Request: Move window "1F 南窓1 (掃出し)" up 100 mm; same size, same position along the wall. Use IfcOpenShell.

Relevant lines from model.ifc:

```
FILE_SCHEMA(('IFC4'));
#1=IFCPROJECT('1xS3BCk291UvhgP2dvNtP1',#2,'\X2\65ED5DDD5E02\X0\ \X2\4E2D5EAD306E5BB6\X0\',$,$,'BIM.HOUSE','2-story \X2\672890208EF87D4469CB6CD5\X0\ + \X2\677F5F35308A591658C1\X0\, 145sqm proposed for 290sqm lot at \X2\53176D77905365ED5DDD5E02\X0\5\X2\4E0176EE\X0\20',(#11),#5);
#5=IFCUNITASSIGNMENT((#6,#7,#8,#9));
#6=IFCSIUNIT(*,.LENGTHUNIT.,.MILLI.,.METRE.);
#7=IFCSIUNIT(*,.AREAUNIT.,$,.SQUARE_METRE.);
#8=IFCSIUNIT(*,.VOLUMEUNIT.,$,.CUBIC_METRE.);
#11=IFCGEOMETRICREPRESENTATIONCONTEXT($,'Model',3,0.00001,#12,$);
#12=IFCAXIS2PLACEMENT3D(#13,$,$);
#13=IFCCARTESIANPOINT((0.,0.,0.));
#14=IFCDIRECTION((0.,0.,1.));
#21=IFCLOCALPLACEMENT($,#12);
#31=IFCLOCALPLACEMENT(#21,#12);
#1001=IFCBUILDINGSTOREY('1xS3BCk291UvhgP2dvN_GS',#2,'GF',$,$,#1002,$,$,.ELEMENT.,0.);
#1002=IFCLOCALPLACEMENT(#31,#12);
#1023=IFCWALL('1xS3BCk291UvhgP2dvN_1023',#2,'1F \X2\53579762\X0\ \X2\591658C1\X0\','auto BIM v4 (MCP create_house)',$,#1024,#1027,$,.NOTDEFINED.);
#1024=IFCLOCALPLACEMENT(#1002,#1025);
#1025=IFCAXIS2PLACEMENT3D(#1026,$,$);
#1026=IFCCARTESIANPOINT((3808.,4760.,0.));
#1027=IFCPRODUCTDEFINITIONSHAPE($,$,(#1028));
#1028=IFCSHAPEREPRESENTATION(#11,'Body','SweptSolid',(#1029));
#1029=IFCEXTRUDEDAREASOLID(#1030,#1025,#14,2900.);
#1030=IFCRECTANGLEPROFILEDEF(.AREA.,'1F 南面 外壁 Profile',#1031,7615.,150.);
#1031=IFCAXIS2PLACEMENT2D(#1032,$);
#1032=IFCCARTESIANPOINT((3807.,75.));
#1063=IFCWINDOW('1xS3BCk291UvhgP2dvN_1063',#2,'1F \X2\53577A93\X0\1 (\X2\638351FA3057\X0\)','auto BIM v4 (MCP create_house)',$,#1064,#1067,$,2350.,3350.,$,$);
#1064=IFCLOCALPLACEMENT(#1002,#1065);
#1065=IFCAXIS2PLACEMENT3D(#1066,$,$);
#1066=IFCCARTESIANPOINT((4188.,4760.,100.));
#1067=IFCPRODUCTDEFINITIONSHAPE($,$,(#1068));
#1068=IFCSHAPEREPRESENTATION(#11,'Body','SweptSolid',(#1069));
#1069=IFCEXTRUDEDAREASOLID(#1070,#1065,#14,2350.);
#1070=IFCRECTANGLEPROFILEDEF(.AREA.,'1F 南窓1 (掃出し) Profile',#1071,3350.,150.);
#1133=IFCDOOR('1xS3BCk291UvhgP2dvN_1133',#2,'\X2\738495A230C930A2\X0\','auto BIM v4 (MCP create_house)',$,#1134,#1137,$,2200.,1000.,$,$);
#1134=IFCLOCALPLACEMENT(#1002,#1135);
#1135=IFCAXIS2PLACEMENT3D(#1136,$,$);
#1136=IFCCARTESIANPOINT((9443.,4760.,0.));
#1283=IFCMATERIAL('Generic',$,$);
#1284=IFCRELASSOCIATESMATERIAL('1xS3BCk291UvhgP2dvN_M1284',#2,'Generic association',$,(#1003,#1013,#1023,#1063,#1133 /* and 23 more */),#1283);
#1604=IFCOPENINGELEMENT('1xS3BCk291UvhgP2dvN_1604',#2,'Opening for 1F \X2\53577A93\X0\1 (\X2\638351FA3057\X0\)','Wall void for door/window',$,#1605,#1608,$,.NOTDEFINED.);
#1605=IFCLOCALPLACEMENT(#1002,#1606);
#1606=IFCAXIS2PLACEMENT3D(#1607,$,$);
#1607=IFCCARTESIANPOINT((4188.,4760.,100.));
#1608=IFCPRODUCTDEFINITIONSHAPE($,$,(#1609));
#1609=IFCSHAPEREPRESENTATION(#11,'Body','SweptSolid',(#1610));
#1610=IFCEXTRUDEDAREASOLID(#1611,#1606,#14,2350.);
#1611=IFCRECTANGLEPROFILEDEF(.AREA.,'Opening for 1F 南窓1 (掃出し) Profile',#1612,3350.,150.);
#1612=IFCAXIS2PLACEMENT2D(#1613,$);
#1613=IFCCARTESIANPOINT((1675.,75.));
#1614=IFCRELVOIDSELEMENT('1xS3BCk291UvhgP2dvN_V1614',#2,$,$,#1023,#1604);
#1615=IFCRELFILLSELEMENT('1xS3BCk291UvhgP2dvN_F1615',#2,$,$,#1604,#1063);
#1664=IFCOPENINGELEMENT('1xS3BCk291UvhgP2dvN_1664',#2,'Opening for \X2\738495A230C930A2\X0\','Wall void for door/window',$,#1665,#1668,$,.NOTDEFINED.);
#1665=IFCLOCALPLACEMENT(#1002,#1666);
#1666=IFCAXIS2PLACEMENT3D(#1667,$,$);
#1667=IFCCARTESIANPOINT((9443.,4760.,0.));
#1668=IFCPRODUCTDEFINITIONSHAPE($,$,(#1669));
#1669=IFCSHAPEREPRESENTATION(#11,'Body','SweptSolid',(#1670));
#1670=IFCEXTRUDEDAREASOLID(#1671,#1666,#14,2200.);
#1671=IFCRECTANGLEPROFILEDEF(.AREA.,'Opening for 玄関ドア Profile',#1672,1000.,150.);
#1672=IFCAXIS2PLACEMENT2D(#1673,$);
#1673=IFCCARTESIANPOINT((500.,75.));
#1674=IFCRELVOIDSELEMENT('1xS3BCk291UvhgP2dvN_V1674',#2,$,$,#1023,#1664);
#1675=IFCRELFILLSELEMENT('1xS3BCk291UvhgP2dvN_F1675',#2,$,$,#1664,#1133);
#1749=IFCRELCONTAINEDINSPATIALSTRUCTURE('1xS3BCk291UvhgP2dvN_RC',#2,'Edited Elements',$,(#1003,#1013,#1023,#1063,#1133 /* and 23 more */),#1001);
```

```python
import numpy as np
import ifcopenshell
import ifcopenshell.api.geometry
import ifcopenshell.util.placement
import ifcopenshell.util.unit

model = ifcopenshell.open("model.ifc")
unit_scale = ifcopenshell.util.unit.calculate_unit_scale(model)

window = model.by_guid("1xS3BCk291UvhgP2dvN_1063")
opening = window.FillsVoids[0].RelatingOpeningElement
dz = 0.1 / unit_scale

shift = np.array([0.0, 0.0, dz])
# The window is not placed relative to its opening, so move both.
for product in (opening, window):
    matrix = ifcopenshell.util.placement.get_local_placement(product.ObjectPlacement)
    matrix[:3, 3] += shift
    ifcopenshell.api.geometry.edit_object_placement(model, product=product, matrix=matrix, is_si=False)

print(f"moved by {dz * unit_scale:+.3f} m")

model.write("model_rev.ifc")
```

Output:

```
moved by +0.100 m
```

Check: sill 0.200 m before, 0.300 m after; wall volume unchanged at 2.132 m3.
